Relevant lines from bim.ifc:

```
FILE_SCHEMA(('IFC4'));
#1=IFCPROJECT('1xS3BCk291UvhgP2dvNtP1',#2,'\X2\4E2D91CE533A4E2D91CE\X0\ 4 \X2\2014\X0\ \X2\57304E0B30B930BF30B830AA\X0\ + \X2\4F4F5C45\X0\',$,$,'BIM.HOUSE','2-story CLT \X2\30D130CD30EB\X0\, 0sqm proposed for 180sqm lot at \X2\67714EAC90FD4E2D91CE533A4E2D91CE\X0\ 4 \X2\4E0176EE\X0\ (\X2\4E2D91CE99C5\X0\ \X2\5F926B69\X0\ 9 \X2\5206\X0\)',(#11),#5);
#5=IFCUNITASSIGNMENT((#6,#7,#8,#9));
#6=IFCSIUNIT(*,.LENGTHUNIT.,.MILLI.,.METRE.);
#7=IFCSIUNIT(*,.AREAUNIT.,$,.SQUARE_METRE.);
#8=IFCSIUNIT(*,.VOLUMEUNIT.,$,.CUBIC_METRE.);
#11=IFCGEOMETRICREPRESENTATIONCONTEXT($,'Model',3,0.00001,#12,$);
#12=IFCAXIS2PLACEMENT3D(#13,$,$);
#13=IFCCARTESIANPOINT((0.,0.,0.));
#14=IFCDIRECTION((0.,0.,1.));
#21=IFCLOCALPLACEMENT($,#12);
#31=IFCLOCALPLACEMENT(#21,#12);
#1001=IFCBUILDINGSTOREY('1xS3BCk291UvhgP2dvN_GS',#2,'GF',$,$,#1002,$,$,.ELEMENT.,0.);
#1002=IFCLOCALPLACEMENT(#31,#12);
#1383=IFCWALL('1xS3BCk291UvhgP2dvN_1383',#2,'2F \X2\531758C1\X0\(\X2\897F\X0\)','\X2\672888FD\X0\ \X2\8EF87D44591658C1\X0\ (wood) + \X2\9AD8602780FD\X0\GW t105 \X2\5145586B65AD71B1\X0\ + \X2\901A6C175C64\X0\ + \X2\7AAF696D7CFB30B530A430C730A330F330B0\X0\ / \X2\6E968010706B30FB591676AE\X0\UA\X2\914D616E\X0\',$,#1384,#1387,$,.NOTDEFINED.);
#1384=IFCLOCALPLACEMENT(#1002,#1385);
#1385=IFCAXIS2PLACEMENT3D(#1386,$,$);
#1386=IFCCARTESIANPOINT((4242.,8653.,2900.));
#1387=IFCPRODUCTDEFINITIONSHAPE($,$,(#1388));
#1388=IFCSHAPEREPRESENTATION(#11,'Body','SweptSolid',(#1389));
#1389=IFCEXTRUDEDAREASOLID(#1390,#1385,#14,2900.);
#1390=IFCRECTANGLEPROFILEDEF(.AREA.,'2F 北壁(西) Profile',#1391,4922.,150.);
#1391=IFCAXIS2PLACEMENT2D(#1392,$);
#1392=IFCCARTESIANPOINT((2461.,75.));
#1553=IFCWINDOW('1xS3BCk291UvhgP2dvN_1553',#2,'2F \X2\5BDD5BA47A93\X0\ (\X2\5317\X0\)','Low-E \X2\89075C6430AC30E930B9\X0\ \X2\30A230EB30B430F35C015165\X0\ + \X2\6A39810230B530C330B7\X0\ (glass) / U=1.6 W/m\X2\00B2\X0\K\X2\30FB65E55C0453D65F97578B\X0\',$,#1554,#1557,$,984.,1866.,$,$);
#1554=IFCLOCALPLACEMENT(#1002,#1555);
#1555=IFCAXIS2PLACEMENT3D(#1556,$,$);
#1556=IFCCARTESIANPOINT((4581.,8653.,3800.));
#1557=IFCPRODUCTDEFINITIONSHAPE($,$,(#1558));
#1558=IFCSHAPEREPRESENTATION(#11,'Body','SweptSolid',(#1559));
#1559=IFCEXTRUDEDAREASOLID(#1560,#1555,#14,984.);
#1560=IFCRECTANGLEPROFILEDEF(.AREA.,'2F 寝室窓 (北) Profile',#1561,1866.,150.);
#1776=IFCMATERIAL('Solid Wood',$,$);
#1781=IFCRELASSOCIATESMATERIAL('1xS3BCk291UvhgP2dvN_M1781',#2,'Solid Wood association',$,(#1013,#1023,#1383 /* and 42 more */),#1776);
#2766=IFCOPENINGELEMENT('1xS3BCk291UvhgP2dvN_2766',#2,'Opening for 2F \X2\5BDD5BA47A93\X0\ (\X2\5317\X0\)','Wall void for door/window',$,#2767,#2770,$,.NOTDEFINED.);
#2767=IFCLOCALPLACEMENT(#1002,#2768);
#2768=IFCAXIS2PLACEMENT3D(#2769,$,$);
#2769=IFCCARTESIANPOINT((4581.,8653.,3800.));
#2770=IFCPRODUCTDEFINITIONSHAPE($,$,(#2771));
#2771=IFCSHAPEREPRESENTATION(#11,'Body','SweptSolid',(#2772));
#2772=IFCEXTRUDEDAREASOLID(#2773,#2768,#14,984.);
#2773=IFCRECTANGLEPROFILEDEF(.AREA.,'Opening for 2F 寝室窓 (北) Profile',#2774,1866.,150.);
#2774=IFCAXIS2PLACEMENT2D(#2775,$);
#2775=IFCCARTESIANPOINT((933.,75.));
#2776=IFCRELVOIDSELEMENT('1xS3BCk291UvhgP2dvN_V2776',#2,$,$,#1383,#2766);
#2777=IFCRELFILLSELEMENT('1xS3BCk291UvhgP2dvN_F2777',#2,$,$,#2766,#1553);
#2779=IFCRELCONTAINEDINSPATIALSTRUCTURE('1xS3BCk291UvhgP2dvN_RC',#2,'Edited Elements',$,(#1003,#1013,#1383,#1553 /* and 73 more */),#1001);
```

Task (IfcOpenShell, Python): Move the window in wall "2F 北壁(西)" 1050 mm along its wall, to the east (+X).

```python
import ifcopenshell
import ifcopenshell.api.geometry
import ifcopenshell.util.placement

model = ifcopenshell.open("bim.ifc")

window = model.by_guid("1xS3BCk291UvhgP2dvN_1553")
opening = window.FillsVoids[0].RelatingOpeningElement
wall = opening.VoidsElements[0].RelatingBuildingElement

wall_matrix = ifcopenshell.util.placement.get_local_placement(wall.ObjectPlacement)
shift = wall_matrix[:3, 0] * 1050.0
before = ifcopenshell.util.placement.get_local_placement(window.ObjectPlacement)[:3, 3].copy()

# The window is not placed relative to its opening, so move both.
for product in (opening, window):
    matrix = ifcopenshell.util.placement.get_local_placement(product.ObjectPlacement)
    matrix[:3, 3] += shift
    ifcopenshell.api.geometry.edit_object_placement(model, product=product, matrix=matrix, is_si=False)

after = ifcopenshell.util.placement.get_local_placement(window.ObjectPlacement)[:3, 3]
print("window moved by", (after - before).round(3) + 0.0)

model.write("bim-out.ifc")
```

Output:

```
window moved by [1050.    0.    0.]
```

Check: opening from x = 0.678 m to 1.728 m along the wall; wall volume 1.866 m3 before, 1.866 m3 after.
